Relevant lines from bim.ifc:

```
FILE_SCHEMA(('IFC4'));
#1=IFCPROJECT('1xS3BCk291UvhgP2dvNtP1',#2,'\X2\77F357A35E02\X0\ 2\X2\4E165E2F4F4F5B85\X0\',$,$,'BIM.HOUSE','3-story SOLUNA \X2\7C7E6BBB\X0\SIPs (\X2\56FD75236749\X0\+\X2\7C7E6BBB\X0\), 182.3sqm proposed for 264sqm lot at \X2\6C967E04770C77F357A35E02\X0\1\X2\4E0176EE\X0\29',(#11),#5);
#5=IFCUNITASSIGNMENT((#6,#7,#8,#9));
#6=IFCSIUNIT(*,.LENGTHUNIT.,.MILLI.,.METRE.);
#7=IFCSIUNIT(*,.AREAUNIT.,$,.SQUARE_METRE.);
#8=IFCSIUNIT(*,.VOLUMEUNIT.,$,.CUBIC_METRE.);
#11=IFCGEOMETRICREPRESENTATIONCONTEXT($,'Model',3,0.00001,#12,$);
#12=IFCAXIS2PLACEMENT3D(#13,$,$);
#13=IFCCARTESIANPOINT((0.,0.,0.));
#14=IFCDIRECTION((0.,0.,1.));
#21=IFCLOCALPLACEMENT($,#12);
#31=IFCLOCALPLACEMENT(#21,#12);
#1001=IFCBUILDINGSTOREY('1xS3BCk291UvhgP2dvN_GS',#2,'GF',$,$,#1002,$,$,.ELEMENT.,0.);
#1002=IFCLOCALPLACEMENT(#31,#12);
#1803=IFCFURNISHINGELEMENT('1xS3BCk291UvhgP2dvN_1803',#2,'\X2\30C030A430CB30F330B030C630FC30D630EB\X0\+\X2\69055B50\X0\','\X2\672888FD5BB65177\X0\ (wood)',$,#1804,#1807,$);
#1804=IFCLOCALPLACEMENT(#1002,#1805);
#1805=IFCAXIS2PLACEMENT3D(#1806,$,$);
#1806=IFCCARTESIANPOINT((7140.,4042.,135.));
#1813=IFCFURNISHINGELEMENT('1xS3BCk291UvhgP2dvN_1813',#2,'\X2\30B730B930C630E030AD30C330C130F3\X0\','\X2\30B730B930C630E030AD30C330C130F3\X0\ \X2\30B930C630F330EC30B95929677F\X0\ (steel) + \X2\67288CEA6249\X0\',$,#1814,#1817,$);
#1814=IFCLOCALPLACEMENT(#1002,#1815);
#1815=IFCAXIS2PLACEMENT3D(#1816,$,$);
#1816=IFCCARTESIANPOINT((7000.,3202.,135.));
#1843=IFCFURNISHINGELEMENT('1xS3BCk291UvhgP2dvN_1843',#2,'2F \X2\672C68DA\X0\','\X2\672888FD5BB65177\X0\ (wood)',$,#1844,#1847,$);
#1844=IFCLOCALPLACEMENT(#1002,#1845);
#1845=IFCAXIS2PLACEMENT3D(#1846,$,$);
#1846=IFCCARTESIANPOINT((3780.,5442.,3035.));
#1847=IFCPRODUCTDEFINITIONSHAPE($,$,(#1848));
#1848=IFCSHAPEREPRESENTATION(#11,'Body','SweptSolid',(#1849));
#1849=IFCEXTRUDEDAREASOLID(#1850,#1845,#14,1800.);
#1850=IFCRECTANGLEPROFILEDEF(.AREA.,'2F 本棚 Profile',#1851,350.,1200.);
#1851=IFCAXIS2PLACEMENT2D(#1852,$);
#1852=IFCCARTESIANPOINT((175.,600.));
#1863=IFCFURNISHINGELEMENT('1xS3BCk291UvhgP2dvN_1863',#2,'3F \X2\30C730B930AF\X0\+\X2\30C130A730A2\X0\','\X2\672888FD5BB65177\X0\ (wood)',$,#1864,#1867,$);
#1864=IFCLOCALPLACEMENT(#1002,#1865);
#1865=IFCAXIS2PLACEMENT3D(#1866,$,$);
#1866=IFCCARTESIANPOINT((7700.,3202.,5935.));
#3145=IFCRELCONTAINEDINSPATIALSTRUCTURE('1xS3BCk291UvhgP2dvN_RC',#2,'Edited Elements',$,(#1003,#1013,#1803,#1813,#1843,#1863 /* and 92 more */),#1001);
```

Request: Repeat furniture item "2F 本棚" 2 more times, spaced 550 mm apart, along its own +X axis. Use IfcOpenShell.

```python
import ifcopenshell
import ifcopenshell.api.geometry
import ifcopenshell.api.root
import ifcopenshell.util.element
import ifcopenshell.util.placement
import ifcopenshell.util.unit

model = ifcopenshell.open("bim.ifc")
unit_scale = ifcopenshell.util.unit.calculate_unit_scale(model)


def reuse_history(source, copy):
    """copy_class also copies each property set's owner history, people and application; keep the originals."""
    for rel in copy.IsDefinedBy:
        if rel.is_a("IfcRelDefinesByProperties") and (history := rel.RelatingPropertyDefinition.OwnerHistory):
            rel.RelatingPropertyDefinition.OwnerHistory = source.OwnerHistory
            ifcopenshell.util.element.remove_deep2(model, history)


source = model.by_guid("1xS3BCk291UvhgP2dvN_1843")
base = ifcopenshell.util.placement.get_local_placement(source.ObjectPlacement)
step = base[:3, 0] * 0.55 / unit_scale

for i in range(1, 3):
    copy = ifcopenshell.api.root.copy_class(model, product=source)
    copy.Representation = ifcopenshell.util.element.copy_deep(
        model, source.Representation, exclude=["IfcGeometricRepresentationContext", "IfcRepresentationMap"]
    )
    reuse_history(source, copy)
    matrix = base.copy()
    matrix[:3, 3] += i * step
    print("added at", matrix[:3, 3].round(3) + 0.0)
    ifcopenshell.api.geometry.edit_object_placement(model, product=copy, matrix=matrix, is_si=False)

model.write("bim-out.ifc")
```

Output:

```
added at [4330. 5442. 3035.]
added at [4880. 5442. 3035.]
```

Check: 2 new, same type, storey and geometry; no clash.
